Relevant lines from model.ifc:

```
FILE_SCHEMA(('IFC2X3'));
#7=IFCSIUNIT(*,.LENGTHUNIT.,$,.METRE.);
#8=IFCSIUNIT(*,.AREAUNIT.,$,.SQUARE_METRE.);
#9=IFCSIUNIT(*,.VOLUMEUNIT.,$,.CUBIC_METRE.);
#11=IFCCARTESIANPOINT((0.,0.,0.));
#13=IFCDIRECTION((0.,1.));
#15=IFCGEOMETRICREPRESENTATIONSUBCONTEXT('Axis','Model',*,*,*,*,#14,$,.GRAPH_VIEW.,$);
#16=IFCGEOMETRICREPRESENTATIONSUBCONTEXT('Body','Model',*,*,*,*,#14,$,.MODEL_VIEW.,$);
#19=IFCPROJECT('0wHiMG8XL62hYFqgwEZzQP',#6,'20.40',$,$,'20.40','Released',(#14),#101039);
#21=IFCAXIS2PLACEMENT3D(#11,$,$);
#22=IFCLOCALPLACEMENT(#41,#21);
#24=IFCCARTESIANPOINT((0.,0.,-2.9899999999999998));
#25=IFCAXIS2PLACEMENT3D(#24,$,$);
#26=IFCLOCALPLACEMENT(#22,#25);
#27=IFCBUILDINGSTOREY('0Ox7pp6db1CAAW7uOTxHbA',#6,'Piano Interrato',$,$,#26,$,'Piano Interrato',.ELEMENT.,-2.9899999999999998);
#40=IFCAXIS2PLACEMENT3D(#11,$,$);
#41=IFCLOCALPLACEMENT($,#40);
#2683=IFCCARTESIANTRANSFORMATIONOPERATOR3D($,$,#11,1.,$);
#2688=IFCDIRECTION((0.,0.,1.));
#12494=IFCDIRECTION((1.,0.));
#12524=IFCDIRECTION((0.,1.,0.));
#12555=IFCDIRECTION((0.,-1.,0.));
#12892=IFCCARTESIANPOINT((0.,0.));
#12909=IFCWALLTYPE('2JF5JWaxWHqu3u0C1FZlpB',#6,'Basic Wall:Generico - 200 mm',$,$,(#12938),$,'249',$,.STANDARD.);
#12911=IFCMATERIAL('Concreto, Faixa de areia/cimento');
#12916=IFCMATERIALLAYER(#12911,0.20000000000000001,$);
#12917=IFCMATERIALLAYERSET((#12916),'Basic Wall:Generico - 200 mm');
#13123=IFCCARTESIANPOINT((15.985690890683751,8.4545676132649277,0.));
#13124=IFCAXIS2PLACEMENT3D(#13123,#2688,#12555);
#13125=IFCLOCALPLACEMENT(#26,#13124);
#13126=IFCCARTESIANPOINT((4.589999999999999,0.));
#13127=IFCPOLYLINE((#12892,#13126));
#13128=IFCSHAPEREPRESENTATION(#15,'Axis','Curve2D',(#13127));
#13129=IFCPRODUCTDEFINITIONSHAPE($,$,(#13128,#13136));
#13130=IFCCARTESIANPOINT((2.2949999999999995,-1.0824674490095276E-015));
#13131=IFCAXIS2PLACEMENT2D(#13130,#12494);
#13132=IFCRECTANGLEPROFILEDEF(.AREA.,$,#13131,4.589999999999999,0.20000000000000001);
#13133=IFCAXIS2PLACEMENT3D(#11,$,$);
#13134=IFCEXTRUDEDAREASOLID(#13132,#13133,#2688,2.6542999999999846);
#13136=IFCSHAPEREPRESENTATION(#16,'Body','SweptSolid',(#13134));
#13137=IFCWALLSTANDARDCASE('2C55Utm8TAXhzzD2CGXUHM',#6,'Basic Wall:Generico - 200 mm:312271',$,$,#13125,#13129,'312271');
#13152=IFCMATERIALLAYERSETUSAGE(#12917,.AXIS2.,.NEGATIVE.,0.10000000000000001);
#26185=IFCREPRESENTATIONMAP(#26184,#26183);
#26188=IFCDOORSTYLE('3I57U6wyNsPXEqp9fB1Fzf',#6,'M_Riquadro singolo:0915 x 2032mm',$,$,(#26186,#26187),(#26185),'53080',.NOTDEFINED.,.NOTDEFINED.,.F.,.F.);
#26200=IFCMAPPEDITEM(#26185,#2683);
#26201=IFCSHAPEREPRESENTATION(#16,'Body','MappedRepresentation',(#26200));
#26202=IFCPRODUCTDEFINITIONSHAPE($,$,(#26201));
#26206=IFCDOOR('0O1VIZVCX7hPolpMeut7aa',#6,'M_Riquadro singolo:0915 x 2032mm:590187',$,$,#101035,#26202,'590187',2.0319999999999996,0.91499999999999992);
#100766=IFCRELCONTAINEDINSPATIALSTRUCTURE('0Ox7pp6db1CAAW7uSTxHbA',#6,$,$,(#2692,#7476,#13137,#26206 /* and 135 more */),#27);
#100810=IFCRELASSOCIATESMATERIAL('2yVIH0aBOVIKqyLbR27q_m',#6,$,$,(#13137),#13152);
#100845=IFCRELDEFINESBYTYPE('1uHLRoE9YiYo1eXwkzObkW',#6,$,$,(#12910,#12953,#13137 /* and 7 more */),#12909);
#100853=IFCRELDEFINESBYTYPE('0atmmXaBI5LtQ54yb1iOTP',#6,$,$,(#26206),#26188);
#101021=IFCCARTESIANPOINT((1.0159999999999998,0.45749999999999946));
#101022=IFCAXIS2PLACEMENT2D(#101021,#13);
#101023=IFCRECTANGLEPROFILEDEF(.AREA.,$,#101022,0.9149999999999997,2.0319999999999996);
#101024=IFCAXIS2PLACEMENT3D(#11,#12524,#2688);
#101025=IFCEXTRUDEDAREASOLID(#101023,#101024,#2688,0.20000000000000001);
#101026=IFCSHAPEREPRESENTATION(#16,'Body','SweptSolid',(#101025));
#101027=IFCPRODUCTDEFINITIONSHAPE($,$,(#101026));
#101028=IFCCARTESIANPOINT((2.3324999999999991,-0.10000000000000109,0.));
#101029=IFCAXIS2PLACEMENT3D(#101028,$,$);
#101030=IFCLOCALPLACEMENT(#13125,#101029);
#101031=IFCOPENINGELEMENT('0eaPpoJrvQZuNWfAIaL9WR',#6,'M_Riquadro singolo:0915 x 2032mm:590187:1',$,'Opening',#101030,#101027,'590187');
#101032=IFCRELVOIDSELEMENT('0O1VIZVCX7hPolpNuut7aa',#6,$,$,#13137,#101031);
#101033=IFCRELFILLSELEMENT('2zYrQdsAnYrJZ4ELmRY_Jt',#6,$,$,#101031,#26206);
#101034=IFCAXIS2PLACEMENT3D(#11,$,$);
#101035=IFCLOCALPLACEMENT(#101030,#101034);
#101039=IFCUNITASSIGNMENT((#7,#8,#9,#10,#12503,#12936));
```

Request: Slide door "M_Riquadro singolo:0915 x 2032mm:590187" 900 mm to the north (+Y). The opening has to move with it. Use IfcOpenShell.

```python
import ifcopenshell
import ifcopenshell.api.geometry
import ifcopenshell.util.placement

model = ifcopenshell.open("model.ifc")

door = model.by_guid("0O1VIZVCX7hPolpMeut7aa")
opening = door.FillsVoids[0].RelatingOpeningElement
wall = opening.VoidsElements[0].RelatingBuildingElement

wall_matrix = ifcopenshell.util.placement.get_local_placement(wall.ObjectPlacement)
shift = wall_matrix[:3, 0] * -0.9
before = ifcopenshell.util.placement.get_local_placement(door.ObjectPlacement)[:3, 3].copy()

# The door is placed relative to its opening, so it follows when the opening moves.
matrix = ifcopenshell.util.placement.get_local_placement(opening.ObjectPlacement)
matrix[:3, 3] += shift
ifcopenshell.api.geometry.edit_object_placement(
    model, product=opening, matrix=matrix, is_si=False, should_transform_children=True
)

after = ifcopenshell.util.placement.get_local_placement(door.ObjectPlacement)[:3, 3]
print("door moved by", (after - before).round(3) + 0.0)

model.write("model-out.ifc")
```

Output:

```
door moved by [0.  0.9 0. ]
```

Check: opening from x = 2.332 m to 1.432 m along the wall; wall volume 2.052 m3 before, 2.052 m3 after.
